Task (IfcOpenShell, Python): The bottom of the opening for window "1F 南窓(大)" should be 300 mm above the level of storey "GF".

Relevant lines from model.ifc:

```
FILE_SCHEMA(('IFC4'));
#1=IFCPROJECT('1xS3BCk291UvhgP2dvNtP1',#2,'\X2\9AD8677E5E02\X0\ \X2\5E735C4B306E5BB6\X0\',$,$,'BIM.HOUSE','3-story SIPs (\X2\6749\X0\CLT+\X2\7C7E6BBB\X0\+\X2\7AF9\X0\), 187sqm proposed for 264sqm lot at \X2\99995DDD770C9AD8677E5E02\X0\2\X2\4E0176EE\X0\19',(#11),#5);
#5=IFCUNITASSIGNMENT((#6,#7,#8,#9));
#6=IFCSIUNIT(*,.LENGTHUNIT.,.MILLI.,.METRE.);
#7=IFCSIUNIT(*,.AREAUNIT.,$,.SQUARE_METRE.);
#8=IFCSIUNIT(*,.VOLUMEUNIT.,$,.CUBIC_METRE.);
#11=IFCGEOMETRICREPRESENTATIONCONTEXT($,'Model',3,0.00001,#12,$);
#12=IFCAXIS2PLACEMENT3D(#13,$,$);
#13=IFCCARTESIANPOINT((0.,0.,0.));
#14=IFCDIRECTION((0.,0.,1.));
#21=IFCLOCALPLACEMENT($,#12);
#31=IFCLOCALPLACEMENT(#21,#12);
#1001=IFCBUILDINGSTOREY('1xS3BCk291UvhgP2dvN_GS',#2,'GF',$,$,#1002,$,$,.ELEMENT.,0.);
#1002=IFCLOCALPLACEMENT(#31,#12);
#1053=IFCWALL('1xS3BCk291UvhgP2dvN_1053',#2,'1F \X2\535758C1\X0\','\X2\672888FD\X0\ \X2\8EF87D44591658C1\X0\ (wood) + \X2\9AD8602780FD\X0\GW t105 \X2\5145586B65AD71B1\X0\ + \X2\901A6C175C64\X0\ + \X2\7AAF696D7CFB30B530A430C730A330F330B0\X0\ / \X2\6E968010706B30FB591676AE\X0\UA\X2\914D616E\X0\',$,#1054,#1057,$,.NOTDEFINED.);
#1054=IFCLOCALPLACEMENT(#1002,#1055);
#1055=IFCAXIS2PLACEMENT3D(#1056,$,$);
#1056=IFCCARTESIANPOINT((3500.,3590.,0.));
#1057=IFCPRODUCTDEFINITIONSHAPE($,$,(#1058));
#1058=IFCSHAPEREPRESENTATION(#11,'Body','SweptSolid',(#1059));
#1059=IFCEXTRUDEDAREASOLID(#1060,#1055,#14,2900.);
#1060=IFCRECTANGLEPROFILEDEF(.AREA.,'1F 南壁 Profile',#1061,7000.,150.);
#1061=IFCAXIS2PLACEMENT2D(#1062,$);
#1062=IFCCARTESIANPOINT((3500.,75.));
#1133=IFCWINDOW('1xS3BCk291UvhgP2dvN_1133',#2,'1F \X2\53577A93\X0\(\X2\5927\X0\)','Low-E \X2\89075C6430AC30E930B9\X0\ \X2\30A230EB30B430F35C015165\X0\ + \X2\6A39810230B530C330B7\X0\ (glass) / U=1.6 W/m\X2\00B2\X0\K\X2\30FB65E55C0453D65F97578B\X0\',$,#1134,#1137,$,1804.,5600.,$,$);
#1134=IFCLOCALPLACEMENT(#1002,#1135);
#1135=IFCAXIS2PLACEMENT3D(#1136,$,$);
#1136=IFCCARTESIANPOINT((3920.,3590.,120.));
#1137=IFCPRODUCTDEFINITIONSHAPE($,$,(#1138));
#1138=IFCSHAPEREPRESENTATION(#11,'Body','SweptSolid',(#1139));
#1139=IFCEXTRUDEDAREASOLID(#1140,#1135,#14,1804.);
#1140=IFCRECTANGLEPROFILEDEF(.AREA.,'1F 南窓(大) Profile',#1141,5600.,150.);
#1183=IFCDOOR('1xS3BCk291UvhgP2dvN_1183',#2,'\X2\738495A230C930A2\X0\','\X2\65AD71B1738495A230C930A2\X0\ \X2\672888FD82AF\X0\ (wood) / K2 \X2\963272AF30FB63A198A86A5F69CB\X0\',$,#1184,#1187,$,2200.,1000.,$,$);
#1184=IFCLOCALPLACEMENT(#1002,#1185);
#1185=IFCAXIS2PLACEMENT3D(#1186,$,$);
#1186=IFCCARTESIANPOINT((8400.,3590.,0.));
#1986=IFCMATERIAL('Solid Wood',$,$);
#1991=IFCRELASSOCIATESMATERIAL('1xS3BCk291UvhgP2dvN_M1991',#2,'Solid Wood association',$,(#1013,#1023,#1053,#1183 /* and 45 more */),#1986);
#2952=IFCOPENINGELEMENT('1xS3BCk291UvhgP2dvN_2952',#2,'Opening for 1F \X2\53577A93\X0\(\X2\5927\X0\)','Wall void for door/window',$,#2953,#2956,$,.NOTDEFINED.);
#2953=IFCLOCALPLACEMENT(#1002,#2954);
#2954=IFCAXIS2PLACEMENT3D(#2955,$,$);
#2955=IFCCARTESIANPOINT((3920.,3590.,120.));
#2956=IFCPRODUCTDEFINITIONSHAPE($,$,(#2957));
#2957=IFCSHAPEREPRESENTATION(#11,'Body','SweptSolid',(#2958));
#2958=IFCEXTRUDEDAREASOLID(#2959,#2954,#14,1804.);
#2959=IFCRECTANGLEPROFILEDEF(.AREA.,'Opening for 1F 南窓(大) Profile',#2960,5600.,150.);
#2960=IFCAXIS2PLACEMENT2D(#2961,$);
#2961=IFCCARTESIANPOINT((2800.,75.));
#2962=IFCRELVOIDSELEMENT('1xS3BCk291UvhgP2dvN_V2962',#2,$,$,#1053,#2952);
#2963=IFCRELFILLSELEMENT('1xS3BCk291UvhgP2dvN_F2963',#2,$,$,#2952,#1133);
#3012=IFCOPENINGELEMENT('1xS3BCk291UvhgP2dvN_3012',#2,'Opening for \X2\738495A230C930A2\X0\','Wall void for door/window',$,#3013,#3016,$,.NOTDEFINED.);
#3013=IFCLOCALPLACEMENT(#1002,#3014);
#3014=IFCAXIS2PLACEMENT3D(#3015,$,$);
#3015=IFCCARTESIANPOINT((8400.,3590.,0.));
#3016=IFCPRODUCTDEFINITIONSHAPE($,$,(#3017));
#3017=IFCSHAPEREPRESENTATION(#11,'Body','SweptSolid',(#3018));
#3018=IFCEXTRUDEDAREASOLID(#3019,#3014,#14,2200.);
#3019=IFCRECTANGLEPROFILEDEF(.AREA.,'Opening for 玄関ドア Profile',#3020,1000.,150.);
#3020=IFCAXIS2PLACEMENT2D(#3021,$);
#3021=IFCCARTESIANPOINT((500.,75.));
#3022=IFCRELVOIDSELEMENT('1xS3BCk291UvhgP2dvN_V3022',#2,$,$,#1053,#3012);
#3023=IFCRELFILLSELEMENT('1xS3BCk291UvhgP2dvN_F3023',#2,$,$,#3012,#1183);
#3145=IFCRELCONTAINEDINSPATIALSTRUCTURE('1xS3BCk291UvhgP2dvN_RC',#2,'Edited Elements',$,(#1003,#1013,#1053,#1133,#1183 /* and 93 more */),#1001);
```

```python
import numpy as np
import ifcopenshell
import ifcopenshell.api.geometry
import ifcopenshell.geom
import ifcopenshell.util.element
import ifcopenshell.util.placement
import ifcopenshell.util.shape
import ifcopenshell.util.unit

model = ifcopenshell.open("model.ifc")
unit_scale = ifcopenshell.util.unit.calculate_unit_scale(model)

window = model.by_guid("1xS3BCk291UvhgP2dvN_1133")
opening = window.FillsVoids[0].RelatingOpeningElement
storey = ifcopenshell.util.element.get_container(window, ifc_class="IfcBuildingStorey")
level = ifcopenshell.util.placement.get_local_placement(storey.ObjectPlacement)[2, 3]

# The opening's origin need not be at the sill, so measure its lowest point.
shape = ifcopenshell.geom.create_shape(ifcopenshell.geom.settings(), opening)
bottom = ifcopenshell.util.shape.get_shape_bottom_elevation(shape, shape.geometry) / unit_scale
dz = level + 300.0 - bottom

shift = np.array([0.0, 0.0, dz])
# The window is not placed relative to its opening, so move both.
for product in (opening, window):
    matrix = ifcopenshell.util.placement.get_local_placement(product.ObjectPlacement)
    matrix[:3, 3] += shift
    ifcopenshell.api.geometry.edit_object_placement(model, product=product, matrix=matrix, is_si=False)

print(f"moved by {dz * unit_scale:+.3f} m")

model.write("model-out.ifc")
```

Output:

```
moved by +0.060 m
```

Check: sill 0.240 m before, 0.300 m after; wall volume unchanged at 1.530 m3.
